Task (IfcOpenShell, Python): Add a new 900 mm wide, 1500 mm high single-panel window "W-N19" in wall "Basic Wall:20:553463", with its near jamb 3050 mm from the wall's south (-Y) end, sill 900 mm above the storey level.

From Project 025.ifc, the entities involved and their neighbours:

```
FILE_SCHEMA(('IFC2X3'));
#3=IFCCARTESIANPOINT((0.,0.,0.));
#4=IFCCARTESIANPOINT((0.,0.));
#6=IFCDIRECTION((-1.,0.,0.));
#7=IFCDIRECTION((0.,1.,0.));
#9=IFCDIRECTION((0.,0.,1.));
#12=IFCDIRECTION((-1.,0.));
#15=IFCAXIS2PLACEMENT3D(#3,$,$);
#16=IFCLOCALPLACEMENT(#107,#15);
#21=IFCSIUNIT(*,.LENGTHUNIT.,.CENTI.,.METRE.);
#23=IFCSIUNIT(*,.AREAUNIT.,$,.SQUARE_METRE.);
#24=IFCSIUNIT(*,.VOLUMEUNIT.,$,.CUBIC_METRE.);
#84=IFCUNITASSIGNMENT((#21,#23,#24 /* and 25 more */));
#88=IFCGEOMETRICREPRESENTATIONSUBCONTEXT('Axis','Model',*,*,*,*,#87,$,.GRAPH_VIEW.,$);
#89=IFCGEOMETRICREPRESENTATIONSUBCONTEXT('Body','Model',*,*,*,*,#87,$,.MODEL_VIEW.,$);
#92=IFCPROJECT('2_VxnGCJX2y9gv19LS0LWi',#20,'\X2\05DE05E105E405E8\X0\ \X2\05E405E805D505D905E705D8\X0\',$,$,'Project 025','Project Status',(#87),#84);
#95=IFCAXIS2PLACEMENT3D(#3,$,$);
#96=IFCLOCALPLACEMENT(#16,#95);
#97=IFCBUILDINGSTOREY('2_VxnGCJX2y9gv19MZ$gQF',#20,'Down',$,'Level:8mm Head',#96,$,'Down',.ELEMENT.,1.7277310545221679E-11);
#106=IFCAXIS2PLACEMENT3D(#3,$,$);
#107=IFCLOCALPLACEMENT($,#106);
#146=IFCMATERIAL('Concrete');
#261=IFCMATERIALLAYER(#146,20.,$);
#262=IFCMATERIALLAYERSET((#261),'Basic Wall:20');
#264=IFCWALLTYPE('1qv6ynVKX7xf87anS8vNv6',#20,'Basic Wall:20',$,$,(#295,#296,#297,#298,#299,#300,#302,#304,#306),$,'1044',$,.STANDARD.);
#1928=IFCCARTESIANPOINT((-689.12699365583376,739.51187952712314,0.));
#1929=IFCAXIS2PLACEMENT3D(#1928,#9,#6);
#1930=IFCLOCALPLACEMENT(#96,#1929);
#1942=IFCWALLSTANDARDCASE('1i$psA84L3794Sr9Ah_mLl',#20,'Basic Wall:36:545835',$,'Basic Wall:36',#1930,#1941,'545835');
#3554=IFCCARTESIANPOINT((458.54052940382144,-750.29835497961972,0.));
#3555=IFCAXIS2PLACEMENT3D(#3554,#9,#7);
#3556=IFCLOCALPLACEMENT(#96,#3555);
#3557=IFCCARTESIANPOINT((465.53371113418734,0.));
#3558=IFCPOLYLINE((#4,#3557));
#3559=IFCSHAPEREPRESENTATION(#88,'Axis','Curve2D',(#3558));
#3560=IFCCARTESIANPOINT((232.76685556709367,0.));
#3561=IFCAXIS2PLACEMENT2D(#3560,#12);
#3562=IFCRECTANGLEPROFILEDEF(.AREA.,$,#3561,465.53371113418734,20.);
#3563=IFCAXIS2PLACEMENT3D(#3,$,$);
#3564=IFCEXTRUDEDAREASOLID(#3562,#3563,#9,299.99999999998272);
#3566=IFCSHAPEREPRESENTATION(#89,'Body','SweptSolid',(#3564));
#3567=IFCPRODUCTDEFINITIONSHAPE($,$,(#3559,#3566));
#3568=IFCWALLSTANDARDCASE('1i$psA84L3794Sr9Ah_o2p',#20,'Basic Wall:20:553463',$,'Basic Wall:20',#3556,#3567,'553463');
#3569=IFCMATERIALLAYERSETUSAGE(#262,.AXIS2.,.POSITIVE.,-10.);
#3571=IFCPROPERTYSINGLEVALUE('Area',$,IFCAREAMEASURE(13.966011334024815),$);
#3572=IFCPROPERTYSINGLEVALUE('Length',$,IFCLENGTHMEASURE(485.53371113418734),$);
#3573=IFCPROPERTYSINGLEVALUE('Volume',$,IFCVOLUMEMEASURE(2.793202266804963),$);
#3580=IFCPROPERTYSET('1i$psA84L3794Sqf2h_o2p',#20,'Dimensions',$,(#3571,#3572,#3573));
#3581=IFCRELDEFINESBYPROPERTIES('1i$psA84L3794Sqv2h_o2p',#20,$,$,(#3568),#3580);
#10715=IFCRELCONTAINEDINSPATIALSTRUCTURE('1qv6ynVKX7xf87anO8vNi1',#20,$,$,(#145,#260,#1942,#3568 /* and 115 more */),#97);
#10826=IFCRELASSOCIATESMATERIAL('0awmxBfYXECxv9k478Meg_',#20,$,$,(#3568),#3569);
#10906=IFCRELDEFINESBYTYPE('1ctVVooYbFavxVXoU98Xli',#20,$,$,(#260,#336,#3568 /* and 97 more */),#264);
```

```python
import numpy as np
import ifcopenshell
import ifcopenshell.api.feature
import ifcopenshell.api.geometry
import ifcopenshell.api.pset
import ifcopenshell.api.root
import ifcopenshell.api.spatial
import ifcopenshell.api.type
import ifcopenshell.geom
import ifcopenshell.util.element
import ifcopenshell.util.placement
import ifcopenshell.util.representation
import ifcopenshell.util.shape
import ifcopenshell.util.unit

model = ifcopenshell.open("Project 025.ifc")
unit_scale = ifcopenshell.util.unit.calculate_unit_scale(model)
area_scale = ifcopenshell.util.unit.calculate_unit_scale(model, "AREAUNIT")
volume_scale = ifcopenshell.util.unit.calculate_unit_scale(model, "VOLUMEUNIT")
settings = ifcopenshell.geom.settings()


def volume(element):
    """Net volume in cubic metres, openings subtracted."""
    shape = ifcopenshell.geom.create_shape(settings, element)
    return ifcopenshell.util.shape.get_volume(shape.geometry)


wall = model.by_guid("1i$psA84L3794Sr9Ah_o2p")
storey = ifcopenshell.util.element.get_container(wall, ifc_class="IfcBuildingStorey")
context = ifcopenshell.util.representation.get_context(model, "Model", "Body", "MODEL_VIEW")
before = volume(wall)

width, height, from_end, sill = 0.9, 1.5, 3.05, 0.9  # metres

# The wall runs along its own X axis, and the end named is its -X end.
wall_shape = ifcopenshell.geom.create_shape(settings, wall)
x, y, z = ifcopenshell.util.shape.get_vertices(wall_shape.geometry).T
start = x.min() + from_end
face, thickness = float(y.min()), float(y.max() - y.min())
wall_matrix = ifcopenshell.util.placement.get_local_placement(wall.ObjectPlacement)
level = ifcopenshell.util.placement.get_local_placement(storey.ObjectPlacement)[2, 3]


def in_wall(x, y):
    """Placement at x, y metres in the wall's axes, at sill height."""
    matrix = wall_matrix.copy()
    matrix[:, 3] = wall_matrix @ np.array([x / unit_scale, y / unit_scale, 0.0, 1.0])
    matrix[2, 3] = level + sill / unit_scale
    return matrix


# Opening: a box that overshoots both wall faces by 50 mm.
opening = ifcopenshell.api.root.create_entity(model, ifc_class="IfcOpeningElement")
box = ifcopenshell.api.geometry.add_wall_representation(
    model, context=context, length=width, height=height, thickness=thickness + 0.1
)
ifcopenshell.api.geometry.assign_representation(model, product=opening, representation=box)
ifcopenshell.api.geometry.edit_object_placement(model, product=opening, matrix=in_wall(start, face - 0.05), is_si=False)
ifcopenshell.api.feature.add_feature(model, feature=opening, element=wall)

window = ifcopenshell.api.root.create_entity(model, ifc_class="IfcWindow", name="W-N19")
window.OverallWidth, window.OverallHeight = width / unit_scale, height / unit_scale
body = ifcopenshell.api.geometry.add_window_representation(
    model,
    context=context,
    overall_width=window.OverallWidth,
    overall_height=window.OverallHeight,
    partition_type="SINGLE_PANEL",
)
ifcopenshell.api.geometry.assign_representation(model, product=window, representation=body)
ifcopenshell.api.spatial.assign_container(model, products=[window], relating_structure=storey)
fills = ifcopenshell.api.feature.add_filling(model, opening=opening, element=window)
fills.OwnerHistory = window.OwnerHistory  # required in IFC2X3

# IFC2X3 keeps the operation on the window style.
style = ifcopenshell.api.root.create_entity(model, ifc_class="IfcWindowStyle", name="W-N19")
style.OperationType, style.ConstructionType = "SINGLE_PANEL", "NOTDEFINED"
style.ParameterTakesPrecedence = style.Sizeable = False
ifcopenshell.api.type.assign_type(model, related_objects=[window], relating_type=style)

# Centre the window in the wall's thickness.
ifcopenshell.api.geometry.edit_object_placement(model, product=window, matrix=in_wall(start, face), is_si=False)
window_shape = ifcopenshell.geom.create_shape(settings, window)
depth = ifcopenshell.util.shape.get_vertices(window_shape.geometry)[:, 1]
offset = face + thickness / 2 - (depth.min() + depth.max()) / 2
ifcopenshell.api.geometry.edit_object_placement(model, product=window, matrix=in_wall(start, offset), is_si=False)

after = volume(wall)

# Update the wall's stored quantities.
pset = model.by_id(ifcopenshell.util.element.get_pset(wall, "Dimensions", should_inherit=False)["id"])
ifcopenshell.api.pset.edit_pset(model, pset=pset, properties={
    "Area": model.create_entity("IfcAreaMeasure", after / thickness / area_scale),
    "Volume": model.create_entity("IfcVolumeMeasure", after / volume_scale),
})

print(f"wall volume {before:.3f} -> {after:.3f} m3")

model.write("Project 025_updated.ifc")
```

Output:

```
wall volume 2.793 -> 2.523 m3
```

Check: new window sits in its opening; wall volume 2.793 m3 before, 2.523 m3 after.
